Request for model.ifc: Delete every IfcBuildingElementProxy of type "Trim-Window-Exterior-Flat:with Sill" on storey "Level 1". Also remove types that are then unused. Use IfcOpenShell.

First a look at what the model holds.

```python
import ifcopenshell
import ifcopenshell.util.element

model = ifcopenshell.open("model.ifc")
print(model.schema)
storey = next(s for s in model.by_type("IfcBuildingStorey") if s.Name == "Level 1")
proxies = [e for e in ifcopenshell.util.element.get_decomposition(storey) if e.is_a("IfcBuildingElementProxy")]
seen = {}
for e in proxies:
    element_type = ifcopenshell.util.element.get_type(e)
    name = element_type.Name if element_type not in (None, e) else None
    seen[name] = seen.get(name, 0) + 1
for name, count in sorted(seen.items(), key=str):
    print(count, "x", name)
```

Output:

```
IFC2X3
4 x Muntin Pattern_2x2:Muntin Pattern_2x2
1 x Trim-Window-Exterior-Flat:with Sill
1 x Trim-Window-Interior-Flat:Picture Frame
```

```python
import ifcopenshell
import ifcopenshell.api.root
import ifcopenshell.util.element

model = ifcopenshell.open("model.ifc")

storey = next(s for s in model.by_type("IfcBuildingStorey") if s.Name == "Level 1")
proxies = [e for e in ifcopenshell.util.element.get_decomposition(storey) if e.is_a("IfcBuildingElementProxy")]
targets = [e for e in proxies if (t := ifcopenshell.util.element.get_type(e)) not in (None, e) and t.Name == "Trim-Window-Exterior-Flat:with Sill"]
types = {ifcopenshell.util.element.get_type(e) for e in targets} - {None, *targets}

for e in targets:
    ifcopenshell.api.root.remove_product(model, product=e)
print(len(targets), "removed")

unused = [t for t in types if not ifcopenshell.util.element.get_types(t)]
for t in unused:
    ifcopenshell.api.root.remove_product(model, product=t)
print(len(unused), "unused types removed")

model.write("model_rev.ifc")
```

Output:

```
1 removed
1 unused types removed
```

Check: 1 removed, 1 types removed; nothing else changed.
